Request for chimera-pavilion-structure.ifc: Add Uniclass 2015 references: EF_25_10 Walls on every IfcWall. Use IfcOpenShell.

First a look at what the model holds.

```python
import ifcopenshell

model = ifcopenshell.open("chimera-pavilion-structure.ifc")
print(model.schema)
print("classifications:", [c.Name for c in model.by_type("IfcClassification")])
for ifc_class in ("IfcDoor", "IfcRoof", "IfcStair", "IfcWall", "IfcWindow"):
    print(ifc_class, len(model.by_type(ifc_class)))
```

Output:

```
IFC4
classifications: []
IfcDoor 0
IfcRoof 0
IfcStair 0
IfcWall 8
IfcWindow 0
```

```python
import ifcopenshell
import ifcopenshell.api.classification

model = ifcopenshell.open("chimera-pavilion-structure.ifc")

system = ifcopenshell.api.classification.add_classification(model, classification="Uniclass 2015")

codes = {
    "IfcWall": ("EF_25_10", "Walls"),
}
for ifc_class, (code, name) in codes.items():
    products = model.by_type(ifc_class)
    ifcopenshell.api.classification.add_reference(
        model, products=products, classification=system, identification=code, name=name
    )
    print(code, len(products))

model.write("chimera-pavilion-structure-out.ifc")
```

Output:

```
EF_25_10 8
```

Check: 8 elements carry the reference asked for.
